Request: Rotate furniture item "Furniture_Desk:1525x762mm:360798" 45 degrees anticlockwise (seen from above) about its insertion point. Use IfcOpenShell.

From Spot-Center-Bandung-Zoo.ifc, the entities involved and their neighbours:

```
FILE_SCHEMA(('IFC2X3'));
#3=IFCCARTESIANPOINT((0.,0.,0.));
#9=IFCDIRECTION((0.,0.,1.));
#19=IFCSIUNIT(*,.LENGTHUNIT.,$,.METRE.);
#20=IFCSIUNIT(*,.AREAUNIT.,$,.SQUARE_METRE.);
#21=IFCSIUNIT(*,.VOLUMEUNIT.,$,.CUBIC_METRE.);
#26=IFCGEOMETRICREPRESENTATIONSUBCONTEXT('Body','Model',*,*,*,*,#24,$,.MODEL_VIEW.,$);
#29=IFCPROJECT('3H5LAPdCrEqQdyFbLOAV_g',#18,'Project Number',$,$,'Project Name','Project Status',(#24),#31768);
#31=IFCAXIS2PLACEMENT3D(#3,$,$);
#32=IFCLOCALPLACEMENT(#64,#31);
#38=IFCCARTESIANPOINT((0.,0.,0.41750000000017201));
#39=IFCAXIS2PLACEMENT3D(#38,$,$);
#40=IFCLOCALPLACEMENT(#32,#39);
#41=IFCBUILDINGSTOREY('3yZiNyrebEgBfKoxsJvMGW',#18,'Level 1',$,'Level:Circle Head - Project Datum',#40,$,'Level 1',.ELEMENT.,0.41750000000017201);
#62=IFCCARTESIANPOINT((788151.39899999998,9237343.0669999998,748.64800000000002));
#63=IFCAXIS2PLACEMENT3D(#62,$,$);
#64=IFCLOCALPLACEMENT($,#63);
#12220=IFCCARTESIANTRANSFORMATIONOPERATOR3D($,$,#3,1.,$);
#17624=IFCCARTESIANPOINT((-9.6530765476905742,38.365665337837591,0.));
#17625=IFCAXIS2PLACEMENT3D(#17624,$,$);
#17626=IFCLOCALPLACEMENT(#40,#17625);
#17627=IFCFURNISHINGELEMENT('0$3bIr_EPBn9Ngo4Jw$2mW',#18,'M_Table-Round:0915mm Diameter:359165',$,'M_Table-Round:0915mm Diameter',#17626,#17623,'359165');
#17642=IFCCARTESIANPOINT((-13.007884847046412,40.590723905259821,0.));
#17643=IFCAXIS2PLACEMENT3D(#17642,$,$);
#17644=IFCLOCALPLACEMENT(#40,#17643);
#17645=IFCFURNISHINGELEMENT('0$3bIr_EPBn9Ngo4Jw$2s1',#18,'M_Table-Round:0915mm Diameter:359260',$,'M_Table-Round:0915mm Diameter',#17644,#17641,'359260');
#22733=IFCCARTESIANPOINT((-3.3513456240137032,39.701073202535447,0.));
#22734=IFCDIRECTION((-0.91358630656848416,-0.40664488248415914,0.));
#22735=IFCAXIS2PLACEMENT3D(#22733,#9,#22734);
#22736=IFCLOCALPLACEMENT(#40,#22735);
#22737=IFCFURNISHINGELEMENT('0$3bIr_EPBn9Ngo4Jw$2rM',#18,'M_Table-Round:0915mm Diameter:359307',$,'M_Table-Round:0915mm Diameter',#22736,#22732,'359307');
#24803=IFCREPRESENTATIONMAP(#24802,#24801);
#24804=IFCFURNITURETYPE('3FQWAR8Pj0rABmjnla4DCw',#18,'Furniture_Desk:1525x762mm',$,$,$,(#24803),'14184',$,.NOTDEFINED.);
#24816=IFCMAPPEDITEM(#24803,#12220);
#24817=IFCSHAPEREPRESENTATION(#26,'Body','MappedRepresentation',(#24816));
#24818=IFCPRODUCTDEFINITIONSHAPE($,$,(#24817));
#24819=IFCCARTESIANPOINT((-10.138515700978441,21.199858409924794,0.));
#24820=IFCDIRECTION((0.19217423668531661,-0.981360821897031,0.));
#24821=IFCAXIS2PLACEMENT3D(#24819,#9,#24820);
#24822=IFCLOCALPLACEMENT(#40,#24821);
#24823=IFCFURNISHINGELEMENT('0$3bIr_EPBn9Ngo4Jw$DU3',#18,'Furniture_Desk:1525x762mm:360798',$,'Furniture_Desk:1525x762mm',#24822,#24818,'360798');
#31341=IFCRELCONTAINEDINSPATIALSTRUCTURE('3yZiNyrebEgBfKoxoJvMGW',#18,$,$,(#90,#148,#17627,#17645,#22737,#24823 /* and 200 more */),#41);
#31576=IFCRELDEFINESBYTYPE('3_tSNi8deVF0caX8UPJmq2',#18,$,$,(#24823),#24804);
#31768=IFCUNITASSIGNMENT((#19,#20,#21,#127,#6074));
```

```python
import ifcopenshell
import ifcopenshell.api.geometry
import ifcopenshell.util.placement

model = ifcopenshell.open("Spot-Center-Bandung-Zoo.ifc")

item = model.by_guid("0$3bIr_EPBn9Ngo4Jw$DU3")
matrix = ifcopenshell.util.placement.get_local_placement(item.ObjectPlacement)
matrix = matrix @ ifcopenshell.util.placement.rotation(45, "Z")
ifcopenshell.api.geometry.edit_object_placement(model, product=item, matrix=matrix, is_si=False)

print(ifcopenshell.util.placement.get_local_placement(item.ObjectPlacement).round(3) + 0.0)

model.write("Spot-Center-Bandung-Zoo_rev.ifc")
```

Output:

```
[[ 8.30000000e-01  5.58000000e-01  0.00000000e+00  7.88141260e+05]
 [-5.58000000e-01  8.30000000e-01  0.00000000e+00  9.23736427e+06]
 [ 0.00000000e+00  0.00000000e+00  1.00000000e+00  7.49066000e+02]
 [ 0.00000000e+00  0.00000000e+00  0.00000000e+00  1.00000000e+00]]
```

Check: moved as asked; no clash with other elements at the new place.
